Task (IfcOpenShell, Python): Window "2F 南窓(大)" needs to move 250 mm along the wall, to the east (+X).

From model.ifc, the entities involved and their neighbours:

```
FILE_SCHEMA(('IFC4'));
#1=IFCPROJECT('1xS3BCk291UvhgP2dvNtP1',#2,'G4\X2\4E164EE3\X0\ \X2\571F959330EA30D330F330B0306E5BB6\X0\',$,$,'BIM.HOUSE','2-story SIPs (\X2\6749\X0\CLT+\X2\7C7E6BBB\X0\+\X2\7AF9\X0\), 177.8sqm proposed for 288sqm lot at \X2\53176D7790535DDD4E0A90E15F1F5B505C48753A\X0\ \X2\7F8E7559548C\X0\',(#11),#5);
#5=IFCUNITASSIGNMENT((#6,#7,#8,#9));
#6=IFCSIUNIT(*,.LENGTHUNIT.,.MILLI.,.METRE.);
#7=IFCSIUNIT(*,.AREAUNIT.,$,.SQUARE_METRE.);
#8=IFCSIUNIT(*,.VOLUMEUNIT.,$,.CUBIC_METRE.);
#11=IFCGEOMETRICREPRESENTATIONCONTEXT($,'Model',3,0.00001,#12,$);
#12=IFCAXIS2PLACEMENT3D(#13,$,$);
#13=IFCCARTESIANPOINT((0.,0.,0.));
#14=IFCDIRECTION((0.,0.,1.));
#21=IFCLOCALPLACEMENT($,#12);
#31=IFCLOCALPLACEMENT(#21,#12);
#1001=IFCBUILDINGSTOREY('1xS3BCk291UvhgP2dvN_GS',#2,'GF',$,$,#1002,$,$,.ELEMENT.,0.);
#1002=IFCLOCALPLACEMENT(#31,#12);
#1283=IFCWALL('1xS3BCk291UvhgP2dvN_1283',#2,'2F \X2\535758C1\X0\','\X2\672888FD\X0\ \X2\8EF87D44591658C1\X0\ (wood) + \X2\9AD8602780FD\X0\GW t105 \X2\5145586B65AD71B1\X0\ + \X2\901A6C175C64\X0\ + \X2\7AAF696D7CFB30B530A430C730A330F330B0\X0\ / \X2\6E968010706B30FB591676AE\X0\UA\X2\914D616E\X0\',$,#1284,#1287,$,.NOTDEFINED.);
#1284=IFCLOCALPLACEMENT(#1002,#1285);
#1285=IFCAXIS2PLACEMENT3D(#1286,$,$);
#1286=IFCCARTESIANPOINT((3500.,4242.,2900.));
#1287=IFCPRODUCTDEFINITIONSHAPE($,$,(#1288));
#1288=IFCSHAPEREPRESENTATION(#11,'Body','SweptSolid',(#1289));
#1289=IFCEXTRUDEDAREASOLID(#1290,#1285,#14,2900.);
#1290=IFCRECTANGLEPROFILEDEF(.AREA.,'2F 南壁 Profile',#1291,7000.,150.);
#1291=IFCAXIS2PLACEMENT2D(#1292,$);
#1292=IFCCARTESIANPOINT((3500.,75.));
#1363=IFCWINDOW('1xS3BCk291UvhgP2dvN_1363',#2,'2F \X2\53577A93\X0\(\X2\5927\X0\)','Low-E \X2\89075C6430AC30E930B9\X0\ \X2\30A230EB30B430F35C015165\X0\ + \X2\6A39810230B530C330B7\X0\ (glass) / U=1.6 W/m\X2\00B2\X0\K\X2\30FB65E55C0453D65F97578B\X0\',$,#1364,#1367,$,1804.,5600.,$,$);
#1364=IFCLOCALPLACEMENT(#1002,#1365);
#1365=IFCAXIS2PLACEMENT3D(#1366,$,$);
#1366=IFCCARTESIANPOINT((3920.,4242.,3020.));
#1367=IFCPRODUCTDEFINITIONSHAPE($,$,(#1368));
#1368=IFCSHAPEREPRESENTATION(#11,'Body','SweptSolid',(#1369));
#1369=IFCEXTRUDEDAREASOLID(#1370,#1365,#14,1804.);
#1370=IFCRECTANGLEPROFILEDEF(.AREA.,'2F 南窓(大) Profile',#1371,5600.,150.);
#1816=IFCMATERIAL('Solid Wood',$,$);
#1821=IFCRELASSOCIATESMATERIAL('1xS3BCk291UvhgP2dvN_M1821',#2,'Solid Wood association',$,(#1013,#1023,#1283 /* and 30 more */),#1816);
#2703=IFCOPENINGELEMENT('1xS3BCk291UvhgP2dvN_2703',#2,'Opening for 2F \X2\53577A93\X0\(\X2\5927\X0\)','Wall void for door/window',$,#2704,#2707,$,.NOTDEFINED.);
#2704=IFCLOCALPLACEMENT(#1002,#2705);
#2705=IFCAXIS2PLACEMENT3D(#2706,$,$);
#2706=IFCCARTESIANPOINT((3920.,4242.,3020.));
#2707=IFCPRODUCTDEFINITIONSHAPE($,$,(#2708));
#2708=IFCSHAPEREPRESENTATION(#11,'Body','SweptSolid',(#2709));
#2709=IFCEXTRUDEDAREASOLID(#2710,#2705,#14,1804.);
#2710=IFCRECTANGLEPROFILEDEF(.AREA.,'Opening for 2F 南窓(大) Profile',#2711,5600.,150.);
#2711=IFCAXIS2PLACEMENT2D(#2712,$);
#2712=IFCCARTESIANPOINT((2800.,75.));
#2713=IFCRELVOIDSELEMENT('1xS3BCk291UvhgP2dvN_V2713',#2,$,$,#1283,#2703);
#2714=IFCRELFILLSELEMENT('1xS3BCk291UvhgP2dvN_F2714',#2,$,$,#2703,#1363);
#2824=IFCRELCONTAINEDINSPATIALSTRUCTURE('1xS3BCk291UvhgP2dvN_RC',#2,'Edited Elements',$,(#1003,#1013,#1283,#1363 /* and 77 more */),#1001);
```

```python
import ifcopenshell
import ifcopenshell.api.geometry
import ifcopenshell.util.placement
import ifcopenshell.util.unit

model = ifcopenshell.open("model.ifc")
unit_scale = ifcopenshell.util.unit.calculate_unit_scale(model)

window = model.by_id(1363)
opening = window.FillsVoids[0].RelatingOpeningElement
wall = opening.VoidsElements[0].RelatingBuildingElement

wall_matrix = ifcopenshell.util.placement.get_local_placement(wall.ObjectPlacement)
shift = wall_matrix[:3, 0] * 0.25 / unit_scale
before = ifcopenshell.util.placement.get_local_placement(window.ObjectPlacement)[:3, 3].copy()

# The window is not placed relative to its opening, so move both.
for product in (opening, window):
    matrix = ifcopenshell.util.placement.get_local_placement(product.ObjectPlacement)
    matrix[:3, 3] += shift
    ifcopenshell.api.geometry.edit_object_placement(model, product=product, matrix=matrix, is_si=False)

after = ifcopenshell.util.placement.get_local_placement(window.ObjectPlacement)[:3, 3]
print("window moved by", (after - before).round(3) + 0.0)

model.write("model_edited.ifc")
```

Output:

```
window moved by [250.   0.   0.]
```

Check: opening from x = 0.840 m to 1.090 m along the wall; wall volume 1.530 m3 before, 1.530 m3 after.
